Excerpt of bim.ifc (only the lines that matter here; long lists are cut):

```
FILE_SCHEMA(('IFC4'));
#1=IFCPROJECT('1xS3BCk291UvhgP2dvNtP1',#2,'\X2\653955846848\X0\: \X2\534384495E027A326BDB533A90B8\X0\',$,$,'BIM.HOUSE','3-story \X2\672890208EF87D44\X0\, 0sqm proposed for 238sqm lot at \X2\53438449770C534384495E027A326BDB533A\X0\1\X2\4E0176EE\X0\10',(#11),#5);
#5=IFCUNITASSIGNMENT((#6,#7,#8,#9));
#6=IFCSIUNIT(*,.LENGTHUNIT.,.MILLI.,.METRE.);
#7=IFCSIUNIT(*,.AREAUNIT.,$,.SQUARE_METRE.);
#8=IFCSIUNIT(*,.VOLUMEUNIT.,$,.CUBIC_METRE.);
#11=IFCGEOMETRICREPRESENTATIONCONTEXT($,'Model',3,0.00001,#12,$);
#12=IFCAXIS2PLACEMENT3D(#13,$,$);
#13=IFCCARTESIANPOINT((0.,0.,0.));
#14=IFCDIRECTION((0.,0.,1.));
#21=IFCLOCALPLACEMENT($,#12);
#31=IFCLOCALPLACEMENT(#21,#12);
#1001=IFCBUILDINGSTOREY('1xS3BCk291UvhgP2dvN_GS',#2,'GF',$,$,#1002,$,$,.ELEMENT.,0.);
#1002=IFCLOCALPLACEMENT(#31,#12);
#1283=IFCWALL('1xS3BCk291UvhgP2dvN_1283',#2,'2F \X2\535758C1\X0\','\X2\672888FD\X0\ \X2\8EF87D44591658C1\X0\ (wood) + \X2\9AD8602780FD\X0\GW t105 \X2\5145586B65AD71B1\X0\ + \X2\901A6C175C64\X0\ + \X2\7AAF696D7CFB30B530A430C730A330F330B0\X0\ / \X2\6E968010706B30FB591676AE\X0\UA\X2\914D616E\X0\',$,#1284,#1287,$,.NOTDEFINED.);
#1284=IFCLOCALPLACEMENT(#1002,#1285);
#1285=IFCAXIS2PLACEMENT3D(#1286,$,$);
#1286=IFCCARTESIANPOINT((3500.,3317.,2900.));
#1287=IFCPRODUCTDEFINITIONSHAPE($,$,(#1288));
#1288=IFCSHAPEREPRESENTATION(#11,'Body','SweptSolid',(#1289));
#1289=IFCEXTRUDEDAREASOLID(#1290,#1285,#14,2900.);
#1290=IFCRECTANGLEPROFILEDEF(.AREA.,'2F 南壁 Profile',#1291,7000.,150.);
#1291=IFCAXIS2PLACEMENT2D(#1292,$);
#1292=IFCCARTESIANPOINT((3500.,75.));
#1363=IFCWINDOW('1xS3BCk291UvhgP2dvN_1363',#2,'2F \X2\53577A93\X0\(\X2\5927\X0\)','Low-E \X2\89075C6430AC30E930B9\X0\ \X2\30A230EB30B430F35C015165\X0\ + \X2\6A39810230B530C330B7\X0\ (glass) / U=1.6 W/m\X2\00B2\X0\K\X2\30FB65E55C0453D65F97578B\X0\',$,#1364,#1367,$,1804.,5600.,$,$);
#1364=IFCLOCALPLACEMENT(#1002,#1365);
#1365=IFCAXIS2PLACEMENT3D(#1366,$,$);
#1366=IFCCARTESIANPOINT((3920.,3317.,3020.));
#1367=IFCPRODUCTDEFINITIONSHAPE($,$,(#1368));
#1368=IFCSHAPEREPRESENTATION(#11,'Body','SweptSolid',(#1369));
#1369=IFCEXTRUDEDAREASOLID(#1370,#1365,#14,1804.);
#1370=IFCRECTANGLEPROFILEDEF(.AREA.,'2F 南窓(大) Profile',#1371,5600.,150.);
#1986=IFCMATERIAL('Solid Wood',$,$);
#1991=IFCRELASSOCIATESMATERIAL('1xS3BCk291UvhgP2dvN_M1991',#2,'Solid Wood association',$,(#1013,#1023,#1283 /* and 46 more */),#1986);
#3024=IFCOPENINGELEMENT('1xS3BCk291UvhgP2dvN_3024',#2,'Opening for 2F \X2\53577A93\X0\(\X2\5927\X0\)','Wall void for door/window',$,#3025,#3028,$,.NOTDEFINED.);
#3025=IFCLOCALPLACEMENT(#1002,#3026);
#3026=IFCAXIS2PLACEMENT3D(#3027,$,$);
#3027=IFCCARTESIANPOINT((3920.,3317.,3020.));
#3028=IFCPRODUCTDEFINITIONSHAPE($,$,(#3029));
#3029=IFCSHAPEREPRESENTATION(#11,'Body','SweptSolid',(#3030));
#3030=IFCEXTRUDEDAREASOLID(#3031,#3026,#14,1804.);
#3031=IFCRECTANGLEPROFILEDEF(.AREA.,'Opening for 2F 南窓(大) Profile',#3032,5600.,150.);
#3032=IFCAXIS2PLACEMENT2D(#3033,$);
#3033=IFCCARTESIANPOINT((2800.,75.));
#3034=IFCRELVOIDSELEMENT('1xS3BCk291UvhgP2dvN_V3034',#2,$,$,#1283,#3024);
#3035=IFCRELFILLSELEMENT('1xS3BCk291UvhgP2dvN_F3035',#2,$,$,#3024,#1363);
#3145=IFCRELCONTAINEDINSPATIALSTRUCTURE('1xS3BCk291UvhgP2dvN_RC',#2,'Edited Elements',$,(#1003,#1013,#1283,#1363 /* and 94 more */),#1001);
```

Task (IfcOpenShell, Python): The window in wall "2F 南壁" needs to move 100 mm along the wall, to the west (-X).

```python
import ifcopenshell
import ifcopenshell.api.geometry
import ifcopenshell.util.placement
import ifcopenshell.util.unit

model = ifcopenshell.open("bim.ifc")
unit_scale = ifcopenshell.util.unit.calculate_unit_scale(model)

window = model.by_guid("1xS3BCk291UvhgP2dvN_1363")
opening = window.FillsVoids[0].RelatingOpeningElement
wall = opening.VoidsElements[0].RelatingBuildingElement

wall_matrix = ifcopenshell.util.placement.get_local_placement(wall.ObjectPlacement)
shift = wall_matrix[:3, 0] * -0.1 / unit_scale
before = ifcopenshell.util.placement.get_local_placement(window.ObjectPlacement)[:3, 3].copy()

# The window is not placed relative to its opening, so move both.
for product in (opening, window):
    matrix = ifcopenshell.util.placement.get_local_placement(product.ObjectPlacement)
    matrix[:3, 3] += shift
    ifcopenshell.api.geometry.edit_object_placement(model, product=product, matrix=matrix, is_si=False)

after = ifcopenshell.util.placement.get_local_placement(window.ObjectPlacement)[:3, 3]
print("window moved by", (after - before).round(3) + 0.0)

model.write("bim_edited.ifc")
```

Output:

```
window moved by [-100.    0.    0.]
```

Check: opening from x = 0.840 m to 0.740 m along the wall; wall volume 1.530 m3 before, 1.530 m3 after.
